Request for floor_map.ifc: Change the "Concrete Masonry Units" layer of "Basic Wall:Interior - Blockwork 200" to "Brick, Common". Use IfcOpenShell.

First a look at what the model holds.

```python
import ifcopenshell
import ifcopenshell.util.element

model = ifcopenshell.open("floor_map.ifc")
print(model.schema)
for layer_set in model.by_type("IfcMaterialLayerSet"):
    if layer_set.LayerSetName == "Basic Wall:Interior - Blockwork 200":
        for layer in layer_set.MaterialLayers:
            print(layer.id(), layer.Material and layer.Material.Name, layer.LayerThickness, sep=" | ")
        print(len(ifcopenshell.util.element.get_elements_by_material(model, layer_set)), "elements and types use it")
print(sorted(m.Name for m in model.by_type("IfcMaterial") if m.Name)[:60])
```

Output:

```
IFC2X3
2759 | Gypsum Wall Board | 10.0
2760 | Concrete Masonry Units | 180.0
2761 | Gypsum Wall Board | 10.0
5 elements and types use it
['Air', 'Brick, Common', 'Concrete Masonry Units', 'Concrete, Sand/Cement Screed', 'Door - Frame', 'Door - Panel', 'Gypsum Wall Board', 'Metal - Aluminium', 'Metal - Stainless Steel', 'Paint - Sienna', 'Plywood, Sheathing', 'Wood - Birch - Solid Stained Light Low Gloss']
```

```python
import ifcopenshell
import ifcopenshell.api.material

model = ifcopenshell.open("floor_map.ifc")

layer_set = next(s for s in model.by_type("IfcMaterialLayerSet") if s.LayerSetName == "Basic Wall:Interior - Blockwork 200")
layer = next(l for l in layer_set.MaterialLayers if l.Material and l.Material.Name == "Concrete Masonry Units")
material = next(m for m in model.by_type("IfcMaterial") if m.Name == "Brick, Common")

# Point this one layer at the other material; renaming the old one would change it everywhere.
ifcopenshell.api.material.edit_layer(model, layer=layer, attributes={}, material=material)

print([l.Material.Name if l.Material else None for l in layer_set.MaterialLayers])

model.write("floor_map_edited.ifc")
```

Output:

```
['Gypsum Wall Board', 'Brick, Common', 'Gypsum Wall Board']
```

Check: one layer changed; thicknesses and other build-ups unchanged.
